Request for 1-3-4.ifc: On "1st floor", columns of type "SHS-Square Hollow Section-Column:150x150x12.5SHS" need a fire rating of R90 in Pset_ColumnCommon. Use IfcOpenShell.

First a look at what the model holds.

```python
import ifcopenshell
import ifcopenshell.util.element

model = ifcopenshell.open("1-3-4.ifc")
print(model.schema)
storey = next(s for s in model.by_type("IfcBuildingStorey") if s.Name == "1st floor")
columns = [e for e in ifcopenshell.util.element.get_decomposition(storey) if e.is_a("IfcColumn")]
seen = {}
for e in columns:
    element_type = ifcopenshell.util.element.get_type(e)
    key = (element_type.Name if element_type != e and element_type else None, ifcopenshell.util.element.get_pset(e, "Pset_ColumnCommon", "FireRating"))
    seen[key] = seen.get(key, 0) + 1
for (name, value), count in sorted(seen.items(), key=str):
    print(count, "x", name, "|", value)
```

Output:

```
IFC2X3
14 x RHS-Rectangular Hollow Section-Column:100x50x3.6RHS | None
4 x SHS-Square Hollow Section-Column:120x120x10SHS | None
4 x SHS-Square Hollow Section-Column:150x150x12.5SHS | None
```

```python
import ifcopenshell
import ifcopenshell.api.pset
import ifcopenshell.util.element

model = ifcopenshell.open("1-3-4.ifc")

storey = next(s for s in model.by_type("IfcBuildingStorey") if s.Name == "1st floor")
columns = [e for e in ifcopenshell.util.element.get_decomposition(storey) if e.is_a("IfcColumn")]

count = 0
for e in columns:
    element_type = ifcopenshell.util.element.get_type(e)
    if element_type in (None, e) or element_type.Name != "SHS-Square Hollow Section-Column:150x150x12.5SHS":
        continue
    # add_pset returns the element's existing set when there is one.
    pset = ifcopenshell.api.pset.add_pset(model, product=e, name="Pset_ColumnCommon")
    ifcopenshell.api.pset.edit_pset(model, pset=pset, properties={"FireRating": "R90"})
    count += 1

print(count, "columns updated")

model.write("1-3-4_updated.ifc")
```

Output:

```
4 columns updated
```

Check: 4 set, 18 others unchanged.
